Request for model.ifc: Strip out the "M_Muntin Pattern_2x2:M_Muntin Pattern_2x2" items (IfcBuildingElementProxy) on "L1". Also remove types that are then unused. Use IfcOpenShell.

First a look at what the model holds.

```python
import ifcopenshell
import ifcopenshell.util.element

model = ifcopenshell.open("model.ifc")
print(model.schema)
storey = next(s for s in model.by_type("IfcBuildingStorey") if s.Name == "L1")
proxies = [e for e in ifcopenshell.util.element.get_decomposition(storey) if e.is_a("IfcBuildingElementProxy")]
seen = {}
for e in proxies:
    element_type = ifcopenshell.util.element.get_type(e)
    name = element_type.Name if element_type not in (None, e) else None
    seen[name] = seen.get(name, 0) + 1
for name, count in sorted(seen.items(), key=str):
    print(count, "x", name)
```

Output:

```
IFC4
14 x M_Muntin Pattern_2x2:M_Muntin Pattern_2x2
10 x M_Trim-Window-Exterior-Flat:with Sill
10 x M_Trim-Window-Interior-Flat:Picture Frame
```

```python
import ifcopenshell
import ifcopenshell.api.root
import ifcopenshell.util.element

model = ifcopenshell.open("model.ifc")

storey = next(s for s in model.by_type("IfcBuildingStorey") if s.Name == "L1")
proxies = [e for e in ifcopenshell.util.element.get_decomposition(storey) if e.is_a("IfcBuildingElementProxy")]
targets = [e for e in proxies if (t := ifcopenshell.util.element.get_type(e)) not in (None, e) and t.Name == "M_Muntin Pattern_2x2:M_Muntin Pattern_2x2"]
types = {ifcopenshell.util.element.get_type(e) for e in targets} - {None, *targets}

for e in targets:
    ifcopenshell.api.root.remove_product(model, product=e)
print(len(targets), "removed")

unused = [t for t in types if not ifcopenshell.util.element.get_types(t)]
for t in unused:
    ifcopenshell.api.root.remove_product(model, product=t)
print(len(unused), "unused types removed")

model.write("model_edited.ifc")
```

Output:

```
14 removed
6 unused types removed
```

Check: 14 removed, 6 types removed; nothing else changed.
